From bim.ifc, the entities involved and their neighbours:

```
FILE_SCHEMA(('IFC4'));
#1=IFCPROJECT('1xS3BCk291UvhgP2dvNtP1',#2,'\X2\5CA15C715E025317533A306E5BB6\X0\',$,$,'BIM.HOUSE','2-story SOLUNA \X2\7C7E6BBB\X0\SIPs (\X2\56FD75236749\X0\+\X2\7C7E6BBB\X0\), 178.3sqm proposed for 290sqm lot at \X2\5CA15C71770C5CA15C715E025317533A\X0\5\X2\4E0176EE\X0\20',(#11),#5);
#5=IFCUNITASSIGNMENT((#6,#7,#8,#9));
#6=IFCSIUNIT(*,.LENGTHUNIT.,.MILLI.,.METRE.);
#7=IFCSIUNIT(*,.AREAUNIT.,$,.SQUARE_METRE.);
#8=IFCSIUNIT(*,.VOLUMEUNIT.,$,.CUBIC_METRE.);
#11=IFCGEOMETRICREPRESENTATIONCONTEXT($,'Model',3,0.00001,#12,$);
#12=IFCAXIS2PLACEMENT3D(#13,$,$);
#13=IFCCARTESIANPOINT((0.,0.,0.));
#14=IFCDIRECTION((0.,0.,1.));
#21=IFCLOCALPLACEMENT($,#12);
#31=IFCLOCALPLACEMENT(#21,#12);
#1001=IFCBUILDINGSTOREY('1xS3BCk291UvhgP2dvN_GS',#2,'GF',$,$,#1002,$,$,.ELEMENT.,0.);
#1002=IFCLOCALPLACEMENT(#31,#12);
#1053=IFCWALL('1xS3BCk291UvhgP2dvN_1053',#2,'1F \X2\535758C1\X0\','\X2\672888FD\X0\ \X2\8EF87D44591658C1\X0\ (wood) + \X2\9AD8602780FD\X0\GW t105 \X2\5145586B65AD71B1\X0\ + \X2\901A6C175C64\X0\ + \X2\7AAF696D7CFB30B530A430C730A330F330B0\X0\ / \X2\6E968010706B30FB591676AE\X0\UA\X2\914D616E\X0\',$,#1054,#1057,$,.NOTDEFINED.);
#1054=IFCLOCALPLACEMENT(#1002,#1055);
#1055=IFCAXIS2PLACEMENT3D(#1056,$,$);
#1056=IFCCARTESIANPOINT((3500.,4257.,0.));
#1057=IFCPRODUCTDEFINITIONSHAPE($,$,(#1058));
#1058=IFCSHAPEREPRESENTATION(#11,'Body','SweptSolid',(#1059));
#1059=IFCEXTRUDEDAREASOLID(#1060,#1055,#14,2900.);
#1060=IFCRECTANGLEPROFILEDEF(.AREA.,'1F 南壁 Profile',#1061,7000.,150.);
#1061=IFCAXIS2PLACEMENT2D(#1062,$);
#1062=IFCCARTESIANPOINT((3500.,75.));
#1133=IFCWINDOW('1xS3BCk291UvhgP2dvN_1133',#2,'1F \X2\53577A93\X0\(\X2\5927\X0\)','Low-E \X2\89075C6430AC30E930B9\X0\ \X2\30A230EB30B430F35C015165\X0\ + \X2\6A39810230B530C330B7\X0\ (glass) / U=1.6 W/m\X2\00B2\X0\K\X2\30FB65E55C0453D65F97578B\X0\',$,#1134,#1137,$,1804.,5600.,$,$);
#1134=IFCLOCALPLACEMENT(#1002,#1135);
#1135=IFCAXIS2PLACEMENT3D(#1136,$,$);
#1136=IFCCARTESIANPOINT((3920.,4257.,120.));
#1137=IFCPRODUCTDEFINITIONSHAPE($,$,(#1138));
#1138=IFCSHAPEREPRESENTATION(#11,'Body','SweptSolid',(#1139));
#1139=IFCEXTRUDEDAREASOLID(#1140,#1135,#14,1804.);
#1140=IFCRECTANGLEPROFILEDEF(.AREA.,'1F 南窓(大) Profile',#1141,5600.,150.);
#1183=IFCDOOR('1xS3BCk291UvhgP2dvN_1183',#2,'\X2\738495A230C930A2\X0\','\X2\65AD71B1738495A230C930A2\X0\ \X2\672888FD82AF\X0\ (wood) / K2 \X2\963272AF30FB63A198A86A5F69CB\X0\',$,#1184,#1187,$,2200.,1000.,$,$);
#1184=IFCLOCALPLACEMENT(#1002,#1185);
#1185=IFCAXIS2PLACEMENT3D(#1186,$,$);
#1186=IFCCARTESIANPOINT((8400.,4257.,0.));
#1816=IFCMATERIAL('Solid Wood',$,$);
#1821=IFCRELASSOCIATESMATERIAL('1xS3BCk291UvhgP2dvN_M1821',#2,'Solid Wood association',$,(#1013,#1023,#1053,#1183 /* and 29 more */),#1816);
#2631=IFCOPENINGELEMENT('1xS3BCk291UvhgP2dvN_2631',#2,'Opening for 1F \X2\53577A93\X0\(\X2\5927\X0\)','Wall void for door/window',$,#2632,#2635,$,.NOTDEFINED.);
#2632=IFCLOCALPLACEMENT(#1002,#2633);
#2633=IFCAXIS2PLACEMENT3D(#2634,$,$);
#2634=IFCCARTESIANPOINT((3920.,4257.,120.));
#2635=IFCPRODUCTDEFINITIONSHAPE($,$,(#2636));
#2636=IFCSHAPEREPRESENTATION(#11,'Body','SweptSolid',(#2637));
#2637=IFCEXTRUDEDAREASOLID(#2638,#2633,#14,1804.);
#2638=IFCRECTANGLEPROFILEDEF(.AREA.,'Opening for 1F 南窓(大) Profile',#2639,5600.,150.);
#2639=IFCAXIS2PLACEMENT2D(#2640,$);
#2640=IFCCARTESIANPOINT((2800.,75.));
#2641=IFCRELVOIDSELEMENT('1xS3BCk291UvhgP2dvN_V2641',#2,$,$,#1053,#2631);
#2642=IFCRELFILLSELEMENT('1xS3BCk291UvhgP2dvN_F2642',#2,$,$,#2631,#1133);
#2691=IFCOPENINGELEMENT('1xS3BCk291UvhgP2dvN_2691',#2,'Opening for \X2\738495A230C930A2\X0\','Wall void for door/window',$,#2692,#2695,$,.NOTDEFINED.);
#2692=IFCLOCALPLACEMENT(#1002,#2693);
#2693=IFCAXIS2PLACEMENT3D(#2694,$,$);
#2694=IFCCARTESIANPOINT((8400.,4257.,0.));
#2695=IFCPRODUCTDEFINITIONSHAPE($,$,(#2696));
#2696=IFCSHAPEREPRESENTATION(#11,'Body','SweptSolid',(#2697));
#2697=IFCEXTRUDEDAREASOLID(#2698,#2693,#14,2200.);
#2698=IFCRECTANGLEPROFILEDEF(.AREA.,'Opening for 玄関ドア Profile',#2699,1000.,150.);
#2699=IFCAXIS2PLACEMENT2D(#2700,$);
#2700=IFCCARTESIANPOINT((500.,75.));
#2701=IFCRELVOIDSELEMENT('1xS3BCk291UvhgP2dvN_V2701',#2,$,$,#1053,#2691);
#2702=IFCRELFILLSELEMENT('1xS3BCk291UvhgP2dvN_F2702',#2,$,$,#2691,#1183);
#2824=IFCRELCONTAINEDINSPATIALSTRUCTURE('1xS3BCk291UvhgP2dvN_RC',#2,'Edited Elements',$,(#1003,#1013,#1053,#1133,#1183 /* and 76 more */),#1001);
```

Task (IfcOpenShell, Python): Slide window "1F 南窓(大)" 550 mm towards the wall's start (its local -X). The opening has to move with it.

```python
import ifcopenshell
import ifcopenshell.api.geometry
import ifcopenshell.util.placement

model = ifcopenshell.open("bim.ifc")

window = model.by_guid("1xS3BCk291UvhgP2dvN_1133")
opening = window.FillsVoids[0].RelatingOpeningElement
wall = opening.VoidsElements[0].RelatingBuildingElement

wall_matrix = ifcopenshell.util.placement.get_local_placement(wall.ObjectPlacement)
shift = wall_matrix[:3, 0] * -550.0
before = ifcopenshell.util.placement.get_local_placement(window.ObjectPlacement)[:3, 3].copy()

# The window is not placed relative to its opening, so move both.
for product in (opening, window):
    matrix = ifcopenshell.util.placement.get_local_placement(product.ObjectPlacement)
    matrix[:3, 3] += shift
    ifcopenshell.api.geometry.edit_object_placement(model, product=product, matrix=matrix, is_si=False)

after = ifcopenshell.util.placement.get_local_placement(window.ObjectPlacement)[:3, 3]
print("window moved by", (after - before).round(3) + 0.0)

model.write("bim_rev.ifc")
```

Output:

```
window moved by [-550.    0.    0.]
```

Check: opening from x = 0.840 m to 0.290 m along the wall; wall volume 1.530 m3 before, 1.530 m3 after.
